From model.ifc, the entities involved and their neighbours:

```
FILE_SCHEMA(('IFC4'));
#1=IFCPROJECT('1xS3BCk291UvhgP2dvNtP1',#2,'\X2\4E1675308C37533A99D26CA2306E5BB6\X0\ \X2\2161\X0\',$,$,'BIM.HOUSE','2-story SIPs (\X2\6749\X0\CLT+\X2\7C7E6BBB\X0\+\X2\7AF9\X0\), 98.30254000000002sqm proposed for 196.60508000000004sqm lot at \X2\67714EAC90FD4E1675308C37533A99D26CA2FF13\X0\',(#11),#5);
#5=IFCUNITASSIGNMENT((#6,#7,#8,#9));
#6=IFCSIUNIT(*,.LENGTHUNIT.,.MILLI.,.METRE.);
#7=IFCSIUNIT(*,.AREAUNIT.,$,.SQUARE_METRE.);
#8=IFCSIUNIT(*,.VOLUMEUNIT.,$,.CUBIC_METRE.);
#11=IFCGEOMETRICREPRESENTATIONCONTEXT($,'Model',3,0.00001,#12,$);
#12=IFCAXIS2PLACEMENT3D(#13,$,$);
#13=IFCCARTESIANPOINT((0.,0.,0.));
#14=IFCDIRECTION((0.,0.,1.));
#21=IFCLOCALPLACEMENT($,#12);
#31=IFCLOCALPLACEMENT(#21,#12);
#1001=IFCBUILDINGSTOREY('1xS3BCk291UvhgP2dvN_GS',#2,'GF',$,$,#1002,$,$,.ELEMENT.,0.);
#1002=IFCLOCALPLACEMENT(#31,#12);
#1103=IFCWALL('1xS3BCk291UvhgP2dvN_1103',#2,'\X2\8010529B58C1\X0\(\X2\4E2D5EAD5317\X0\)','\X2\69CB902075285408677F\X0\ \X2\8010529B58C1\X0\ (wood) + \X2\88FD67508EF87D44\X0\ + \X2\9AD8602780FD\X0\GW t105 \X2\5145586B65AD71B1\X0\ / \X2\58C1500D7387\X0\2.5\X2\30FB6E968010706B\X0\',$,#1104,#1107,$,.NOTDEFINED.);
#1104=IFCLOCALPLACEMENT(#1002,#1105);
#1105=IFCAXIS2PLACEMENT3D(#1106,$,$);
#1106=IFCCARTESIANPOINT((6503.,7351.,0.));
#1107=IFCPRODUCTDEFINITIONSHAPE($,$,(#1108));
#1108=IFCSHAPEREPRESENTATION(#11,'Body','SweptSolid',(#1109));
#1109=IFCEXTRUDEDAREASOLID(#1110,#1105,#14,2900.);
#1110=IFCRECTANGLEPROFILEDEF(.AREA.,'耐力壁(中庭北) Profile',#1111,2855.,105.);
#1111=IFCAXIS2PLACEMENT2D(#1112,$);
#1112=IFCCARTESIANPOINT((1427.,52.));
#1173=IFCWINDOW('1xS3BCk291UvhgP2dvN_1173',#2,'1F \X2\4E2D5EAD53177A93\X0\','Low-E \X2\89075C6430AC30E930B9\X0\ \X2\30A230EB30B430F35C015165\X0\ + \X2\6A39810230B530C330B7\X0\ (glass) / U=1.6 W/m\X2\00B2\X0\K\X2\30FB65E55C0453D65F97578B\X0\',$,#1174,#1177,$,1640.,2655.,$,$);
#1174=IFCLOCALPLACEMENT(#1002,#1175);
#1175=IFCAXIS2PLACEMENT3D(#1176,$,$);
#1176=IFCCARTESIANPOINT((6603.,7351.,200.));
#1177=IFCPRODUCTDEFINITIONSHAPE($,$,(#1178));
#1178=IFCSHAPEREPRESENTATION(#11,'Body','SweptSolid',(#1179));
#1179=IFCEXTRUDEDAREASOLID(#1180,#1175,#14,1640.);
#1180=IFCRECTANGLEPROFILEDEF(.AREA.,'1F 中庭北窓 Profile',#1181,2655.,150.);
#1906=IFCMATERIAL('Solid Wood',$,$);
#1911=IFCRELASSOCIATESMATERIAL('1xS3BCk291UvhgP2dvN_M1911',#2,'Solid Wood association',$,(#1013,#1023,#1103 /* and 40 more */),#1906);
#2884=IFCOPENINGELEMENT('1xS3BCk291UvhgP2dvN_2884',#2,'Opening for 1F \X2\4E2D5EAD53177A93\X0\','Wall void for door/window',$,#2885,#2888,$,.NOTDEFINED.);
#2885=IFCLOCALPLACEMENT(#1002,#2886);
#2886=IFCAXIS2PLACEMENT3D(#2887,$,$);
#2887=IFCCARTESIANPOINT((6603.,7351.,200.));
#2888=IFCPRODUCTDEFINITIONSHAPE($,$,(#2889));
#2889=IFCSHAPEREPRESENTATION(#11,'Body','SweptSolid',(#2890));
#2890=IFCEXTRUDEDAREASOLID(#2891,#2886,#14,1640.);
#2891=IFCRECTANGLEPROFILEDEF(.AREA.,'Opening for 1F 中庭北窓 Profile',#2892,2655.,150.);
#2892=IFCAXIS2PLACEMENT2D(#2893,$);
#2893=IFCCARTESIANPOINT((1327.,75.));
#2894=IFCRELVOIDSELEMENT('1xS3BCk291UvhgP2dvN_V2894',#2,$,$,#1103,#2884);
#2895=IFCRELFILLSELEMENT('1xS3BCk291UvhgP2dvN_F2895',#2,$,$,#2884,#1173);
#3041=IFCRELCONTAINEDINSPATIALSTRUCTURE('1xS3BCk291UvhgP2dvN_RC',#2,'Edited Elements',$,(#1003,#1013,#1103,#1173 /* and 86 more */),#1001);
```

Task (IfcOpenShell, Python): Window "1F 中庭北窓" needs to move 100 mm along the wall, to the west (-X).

```python
import ifcopenshell
import ifcopenshell.api.geometry
import ifcopenshell.util.placement
import ifcopenshell.util.unit

model = ifcopenshell.open("model.ifc")
unit_scale = ifcopenshell.util.unit.calculate_unit_scale(model)

window = model.by_id(1173)
opening = window.FillsVoids[0].RelatingOpeningElement
wall = opening.VoidsElements[0].RelatingBuildingElement

wall_matrix = ifcopenshell.util.placement.get_local_placement(wall.ObjectPlacement)
shift = wall_matrix[:3, 0] * -0.1 / unit_scale
before = ifcopenshell.util.placement.get_local_placement(window.ObjectPlacement)[:3, 3].copy()

# The window is not placed relative to its opening, so move both.
for product in (opening, window):
    matrix = ifcopenshell.util.placement.get_local_placement(product.ObjectPlacement)
    matrix[:3, 3] += shift
    ifcopenshell.api.geometry.edit_object_placement(model, product=product, matrix=matrix, is_si=False)

after = ifcopenshell.util.placement.get_local_placement(window.ObjectPlacement)[:3, 3]
print("window moved by", (after - before).round(3) + 0.0)

model.write("model_rev.ifc")
```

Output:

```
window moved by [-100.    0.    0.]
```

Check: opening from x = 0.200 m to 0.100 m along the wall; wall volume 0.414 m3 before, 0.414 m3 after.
